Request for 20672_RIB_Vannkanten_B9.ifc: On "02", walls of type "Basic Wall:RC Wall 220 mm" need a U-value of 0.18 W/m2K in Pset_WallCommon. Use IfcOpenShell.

First a look at what the model holds.

```python
import ifcopenshell
import ifcopenshell.util.element

model = ifcopenshell.open("20672_RIB_Vannkanten_B9.ifc")
print(model.schema)
storey = next(s for s in model.by_type("IfcBuildingStorey") if s.Name == "02")
walls = [e for e in ifcopenshell.util.element.get_decomposition(storey) if e.is_a("IfcWall")]
seen = {}
for e in walls:
    element_type = ifcopenshell.util.element.get_type(e)
    key = (element_type.Name if element_type != e and element_type else None, ifcopenshell.util.element.get_pset(e, "Pset_WallCommon", "ThermalTransmittance"))
    seen[key] = seen.get(key, 0) + 1
for (name, value), count in sorted(seen.items(), key=str):
    print(count, "x", name, "|", value)
```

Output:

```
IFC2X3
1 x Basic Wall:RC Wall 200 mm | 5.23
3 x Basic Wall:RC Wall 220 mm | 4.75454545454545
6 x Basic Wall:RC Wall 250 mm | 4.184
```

```python
import ifcopenshell
import ifcopenshell.api.pset
import ifcopenshell.util.element

model = ifcopenshell.open("20672_RIB_Vannkanten_B9.ifc")

storey = next(s for s in model.by_type("IfcBuildingStorey") if s.Name == "02")
walls = [e for e in ifcopenshell.util.element.get_decomposition(storey) if e.is_a("IfcWall")]

count = 0
for e in walls:
    element_type = ifcopenshell.util.element.get_type(e)
    if element_type in (None, e) or element_type.Name != "Basic Wall:RC Wall 220 mm":
        continue
    # add_pset returns the element's existing set when there is one.
    pset = ifcopenshell.api.pset.add_pset(model, product=e, name="Pset_WallCommon")
    ifcopenshell.api.pset.edit_pset(model, pset=pset, properties={"ThermalTransmittance": 0.18})
    count += 1

print(count, "walls updated")

model.write("20672_RIB_Vannkanten_B9_v2.ifc")
```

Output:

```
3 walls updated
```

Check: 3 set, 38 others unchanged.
